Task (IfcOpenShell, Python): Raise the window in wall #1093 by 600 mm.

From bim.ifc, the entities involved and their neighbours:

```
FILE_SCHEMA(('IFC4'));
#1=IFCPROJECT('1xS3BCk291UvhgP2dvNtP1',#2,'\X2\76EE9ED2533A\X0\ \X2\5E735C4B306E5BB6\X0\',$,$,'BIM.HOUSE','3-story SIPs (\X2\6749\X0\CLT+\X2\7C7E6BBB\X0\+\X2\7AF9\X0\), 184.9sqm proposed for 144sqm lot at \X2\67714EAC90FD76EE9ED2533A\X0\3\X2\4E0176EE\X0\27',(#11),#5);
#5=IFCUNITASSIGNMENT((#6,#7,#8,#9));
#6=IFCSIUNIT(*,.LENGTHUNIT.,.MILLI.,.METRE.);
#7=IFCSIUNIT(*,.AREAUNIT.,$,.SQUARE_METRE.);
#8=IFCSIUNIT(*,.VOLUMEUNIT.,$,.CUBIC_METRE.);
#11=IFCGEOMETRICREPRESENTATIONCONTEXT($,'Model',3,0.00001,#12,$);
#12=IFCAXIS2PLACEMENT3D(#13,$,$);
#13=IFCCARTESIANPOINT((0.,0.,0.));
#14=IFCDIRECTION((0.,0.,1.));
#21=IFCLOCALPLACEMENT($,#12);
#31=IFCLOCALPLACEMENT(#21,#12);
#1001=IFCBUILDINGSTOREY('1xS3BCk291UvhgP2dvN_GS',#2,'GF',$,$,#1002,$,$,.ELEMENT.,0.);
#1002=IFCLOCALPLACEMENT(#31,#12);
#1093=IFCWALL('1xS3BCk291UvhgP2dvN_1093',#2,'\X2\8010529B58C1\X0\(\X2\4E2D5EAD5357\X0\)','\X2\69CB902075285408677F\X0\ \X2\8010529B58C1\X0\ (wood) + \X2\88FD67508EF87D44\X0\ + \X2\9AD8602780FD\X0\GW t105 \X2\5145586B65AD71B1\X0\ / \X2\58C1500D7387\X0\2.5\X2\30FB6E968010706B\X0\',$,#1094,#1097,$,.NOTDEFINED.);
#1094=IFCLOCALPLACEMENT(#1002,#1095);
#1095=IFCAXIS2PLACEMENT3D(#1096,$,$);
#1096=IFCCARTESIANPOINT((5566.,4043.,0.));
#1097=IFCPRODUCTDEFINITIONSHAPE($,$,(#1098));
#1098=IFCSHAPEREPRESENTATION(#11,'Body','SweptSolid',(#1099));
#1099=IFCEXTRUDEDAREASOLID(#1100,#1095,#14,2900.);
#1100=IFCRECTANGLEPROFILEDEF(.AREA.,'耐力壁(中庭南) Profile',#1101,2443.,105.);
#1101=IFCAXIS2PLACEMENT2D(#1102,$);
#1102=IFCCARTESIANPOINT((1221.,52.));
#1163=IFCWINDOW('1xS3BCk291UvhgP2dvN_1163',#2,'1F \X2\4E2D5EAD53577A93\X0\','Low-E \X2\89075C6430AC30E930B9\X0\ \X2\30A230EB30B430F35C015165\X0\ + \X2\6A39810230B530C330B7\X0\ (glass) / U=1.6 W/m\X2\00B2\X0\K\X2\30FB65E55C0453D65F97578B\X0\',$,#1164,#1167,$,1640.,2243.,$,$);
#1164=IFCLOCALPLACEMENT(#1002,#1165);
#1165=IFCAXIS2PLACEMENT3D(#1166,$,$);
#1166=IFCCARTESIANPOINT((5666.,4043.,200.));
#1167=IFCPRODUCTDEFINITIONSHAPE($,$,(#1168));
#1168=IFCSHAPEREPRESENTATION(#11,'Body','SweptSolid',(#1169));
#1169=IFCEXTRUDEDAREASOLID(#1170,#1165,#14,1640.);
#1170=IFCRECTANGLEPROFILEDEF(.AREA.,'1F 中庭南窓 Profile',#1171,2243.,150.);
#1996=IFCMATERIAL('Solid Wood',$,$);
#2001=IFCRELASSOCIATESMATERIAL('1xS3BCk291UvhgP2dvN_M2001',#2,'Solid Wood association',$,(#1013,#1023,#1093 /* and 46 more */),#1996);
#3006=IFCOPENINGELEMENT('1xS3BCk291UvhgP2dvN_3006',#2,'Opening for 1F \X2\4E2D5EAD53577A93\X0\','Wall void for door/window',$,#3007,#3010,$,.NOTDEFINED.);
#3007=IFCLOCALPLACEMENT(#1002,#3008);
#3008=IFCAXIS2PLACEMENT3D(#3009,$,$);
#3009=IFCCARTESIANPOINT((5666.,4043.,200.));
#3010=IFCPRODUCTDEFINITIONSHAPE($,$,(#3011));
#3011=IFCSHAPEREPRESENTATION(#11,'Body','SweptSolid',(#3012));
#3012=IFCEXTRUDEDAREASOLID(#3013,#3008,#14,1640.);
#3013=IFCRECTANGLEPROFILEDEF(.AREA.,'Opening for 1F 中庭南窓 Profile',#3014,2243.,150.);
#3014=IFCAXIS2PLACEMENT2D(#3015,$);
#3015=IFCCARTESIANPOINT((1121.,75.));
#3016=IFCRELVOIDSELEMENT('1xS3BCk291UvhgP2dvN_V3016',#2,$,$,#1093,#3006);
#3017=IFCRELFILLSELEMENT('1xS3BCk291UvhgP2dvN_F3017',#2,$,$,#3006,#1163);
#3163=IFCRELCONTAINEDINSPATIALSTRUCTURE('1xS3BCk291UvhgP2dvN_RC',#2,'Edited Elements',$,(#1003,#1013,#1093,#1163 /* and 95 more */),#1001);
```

```python
import numpy as np
import ifcopenshell
import ifcopenshell.api.geometry
import ifcopenshell.util.placement
import ifcopenshell.util.unit

model = ifcopenshell.open("bim.ifc")
unit_scale = ifcopenshell.util.unit.calculate_unit_scale(model)

window = model.by_guid("1xS3BCk291UvhgP2dvN_1163")
opening = window.FillsVoids[0].RelatingOpeningElement
dz = 600.0

shift = np.array([0.0, 0.0, dz])
# The window is not placed relative to its opening, so move both.
for product in (opening, window):
    matrix = ifcopenshell.util.placement.get_local_placement(product.ObjectPlacement)
    matrix[:3, 3] += shift
    ifcopenshell.api.geometry.edit_object_placement(model, product=product, matrix=matrix, is_si=False)

print(f"moved by {dz * unit_scale:+.3f} m")

model.write("bim_rev.ifc")
```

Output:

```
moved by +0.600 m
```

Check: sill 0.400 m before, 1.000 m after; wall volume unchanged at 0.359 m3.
